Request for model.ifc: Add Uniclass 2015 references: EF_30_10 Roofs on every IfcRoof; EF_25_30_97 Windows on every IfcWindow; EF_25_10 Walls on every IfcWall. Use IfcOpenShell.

First a look at what the model holds.

```python
import ifcopenshell

model = ifcopenshell.open("model.ifc")
print(model.schema)
print("classifications:", [c.Name for c in model.by_type("IfcClassification")])
for ifc_class in ("IfcDoor", "IfcRoof", "IfcStair", "IfcWall", "IfcWindow"):
    print(ifc_class, len(model.by_type(ifc_class)))
```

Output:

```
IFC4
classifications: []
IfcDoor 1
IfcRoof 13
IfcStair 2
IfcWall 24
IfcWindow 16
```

```python
import ifcopenshell
import ifcopenshell.api.classification

model = ifcopenshell.open("model.ifc")

system = ifcopenshell.api.classification.add_classification(model, classification="Uniclass 2015")

codes = {
    "IfcRoof": ("EF_30_10", "Roofs"),
    "IfcWindow": ("EF_25_30_97", "Windows"),
    "IfcWall": ("EF_25_10", "Walls"),
}
for ifc_class, (code, name) in codes.items():
    products = model.by_type(ifc_class)
    ifcopenshell.api.classification.add_reference(
        model, products=products, classification=system, identification=code, name=name
    )
    print(code, len(products))

model.write("model_v2.ifc")
```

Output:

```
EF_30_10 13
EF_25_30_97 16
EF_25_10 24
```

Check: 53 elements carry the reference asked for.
